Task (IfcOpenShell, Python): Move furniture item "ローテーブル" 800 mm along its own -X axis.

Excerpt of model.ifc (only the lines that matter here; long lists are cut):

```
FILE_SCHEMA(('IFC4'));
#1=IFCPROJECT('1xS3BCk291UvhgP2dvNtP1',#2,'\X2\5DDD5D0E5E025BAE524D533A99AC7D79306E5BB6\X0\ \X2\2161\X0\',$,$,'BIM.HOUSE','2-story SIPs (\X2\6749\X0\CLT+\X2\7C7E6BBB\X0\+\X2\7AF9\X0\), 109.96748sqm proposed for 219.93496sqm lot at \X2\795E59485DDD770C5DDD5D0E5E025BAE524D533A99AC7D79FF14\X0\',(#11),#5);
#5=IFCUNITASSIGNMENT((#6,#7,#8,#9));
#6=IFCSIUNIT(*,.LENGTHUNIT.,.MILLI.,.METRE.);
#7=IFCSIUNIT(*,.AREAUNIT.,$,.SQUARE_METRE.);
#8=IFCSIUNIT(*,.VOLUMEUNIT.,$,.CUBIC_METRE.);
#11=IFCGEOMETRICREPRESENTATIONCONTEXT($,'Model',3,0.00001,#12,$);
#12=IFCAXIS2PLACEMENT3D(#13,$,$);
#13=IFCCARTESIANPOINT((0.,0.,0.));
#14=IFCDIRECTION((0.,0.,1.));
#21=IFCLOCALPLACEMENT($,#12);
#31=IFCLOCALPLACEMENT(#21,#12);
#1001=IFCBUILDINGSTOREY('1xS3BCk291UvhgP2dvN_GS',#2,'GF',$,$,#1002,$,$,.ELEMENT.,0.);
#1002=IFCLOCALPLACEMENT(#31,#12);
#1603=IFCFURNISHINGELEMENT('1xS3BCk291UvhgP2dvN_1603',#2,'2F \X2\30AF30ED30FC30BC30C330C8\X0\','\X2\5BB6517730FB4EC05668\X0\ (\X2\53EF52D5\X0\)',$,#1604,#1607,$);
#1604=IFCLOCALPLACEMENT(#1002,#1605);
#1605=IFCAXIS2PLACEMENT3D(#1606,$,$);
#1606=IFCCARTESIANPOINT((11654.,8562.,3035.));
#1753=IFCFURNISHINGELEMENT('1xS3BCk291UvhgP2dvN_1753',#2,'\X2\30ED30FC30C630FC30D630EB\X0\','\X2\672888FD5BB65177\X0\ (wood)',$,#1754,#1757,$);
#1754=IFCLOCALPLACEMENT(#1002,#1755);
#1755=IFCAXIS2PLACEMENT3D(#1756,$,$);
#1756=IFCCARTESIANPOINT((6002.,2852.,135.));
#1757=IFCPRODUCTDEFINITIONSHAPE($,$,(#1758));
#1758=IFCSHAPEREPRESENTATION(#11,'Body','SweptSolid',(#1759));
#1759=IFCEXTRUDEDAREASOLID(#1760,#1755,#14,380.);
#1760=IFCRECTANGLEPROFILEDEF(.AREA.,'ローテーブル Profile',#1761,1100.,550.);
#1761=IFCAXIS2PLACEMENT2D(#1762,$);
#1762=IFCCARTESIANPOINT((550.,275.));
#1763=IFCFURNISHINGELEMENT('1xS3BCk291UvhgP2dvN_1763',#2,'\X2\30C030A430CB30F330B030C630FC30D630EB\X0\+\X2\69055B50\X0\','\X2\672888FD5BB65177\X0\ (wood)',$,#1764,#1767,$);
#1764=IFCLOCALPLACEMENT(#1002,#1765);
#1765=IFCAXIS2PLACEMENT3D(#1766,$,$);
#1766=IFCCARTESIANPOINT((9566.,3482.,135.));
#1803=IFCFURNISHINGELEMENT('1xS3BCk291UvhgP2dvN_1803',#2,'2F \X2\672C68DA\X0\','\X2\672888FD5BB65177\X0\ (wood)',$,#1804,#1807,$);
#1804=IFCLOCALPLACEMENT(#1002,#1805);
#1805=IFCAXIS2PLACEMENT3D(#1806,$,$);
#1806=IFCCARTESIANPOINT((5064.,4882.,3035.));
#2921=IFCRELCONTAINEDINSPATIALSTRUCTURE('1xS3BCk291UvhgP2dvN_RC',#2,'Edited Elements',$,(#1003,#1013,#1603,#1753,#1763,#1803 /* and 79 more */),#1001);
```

```python
import ifcopenshell
import ifcopenshell.api.geometry
import ifcopenshell.util.placement
import ifcopenshell.util.unit

model = ifcopenshell.open("model.ifc")
unit_scale = ifcopenshell.util.unit.calculate_unit_scale(model)

item = model.by_guid("1xS3BCk291UvhgP2dvN_1753")
matrix = ifcopenshell.util.placement.get_local_placement(item.ObjectPlacement)
matrix[:3, 3] -= matrix[:3, 0] * 0.8 / unit_scale
ifcopenshell.api.geometry.edit_object_placement(model, product=item, matrix=matrix, is_si=False)

print(ifcopenshell.util.placement.get_local_placement(item.ObjectPlacement).round(3) + 0.0)

model.write("model_edited.ifc")
```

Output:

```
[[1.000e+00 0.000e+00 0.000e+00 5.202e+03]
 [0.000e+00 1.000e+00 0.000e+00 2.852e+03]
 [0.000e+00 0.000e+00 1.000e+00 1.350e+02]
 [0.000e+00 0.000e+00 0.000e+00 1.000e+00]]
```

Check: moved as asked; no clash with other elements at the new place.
